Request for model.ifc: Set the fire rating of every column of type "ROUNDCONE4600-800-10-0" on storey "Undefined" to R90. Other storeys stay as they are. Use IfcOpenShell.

First a look at what the model holds.

```python
import ifcopenshell
import ifcopenshell.util.element

model = ifcopenshell.open("model.ifc")
print(model.schema)
storey = next(s for s in model.by_type("IfcBuildingStorey") if s.Name == "Undefined")
columns = [e for e in ifcopenshell.util.element.get_decomposition(storey) if e.is_a("IfcColumn")]
seen = {}
for e in columns:
    element_type = ifcopenshell.util.element.get_type(e)
    key = (element_type.Name if element_type != e and element_type else None, ifcopenshell.util.element.get_pset(e, "Pset_ColumnCommon", "FireRating"))
    seen[key] = seen.get(key, 0) + 1
for (name, value), count in sorted(seen.items(), key=str):
    print(count, "x", name, "|", value)
```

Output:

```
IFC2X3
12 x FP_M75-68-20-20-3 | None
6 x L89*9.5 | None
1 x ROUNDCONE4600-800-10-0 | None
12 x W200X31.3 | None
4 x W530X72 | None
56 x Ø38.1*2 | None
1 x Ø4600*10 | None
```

```python
import ifcopenshell
import ifcopenshell.api.pset
import ifcopenshell.util.element

model = ifcopenshell.open("model.ifc")

storey = next(s for s in model.by_type("IfcBuildingStorey") if s.Name == "Undefined")
columns = [e for e in ifcopenshell.util.element.get_decomposition(storey) if e.is_a("IfcColumn")]

count = 0
for e in columns:
    element_type = ifcopenshell.util.element.get_type(e)
    if element_type in (None, e) or element_type.Name != "ROUNDCONE4600-800-10-0":
        continue
    # add_pset returns the element's existing set when there is one.
    pset = ifcopenshell.api.pset.add_pset(model, product=e, name="Pset_ColumnCommon")
    ifcopenshell.api.pset.edit_pset(model, pset=pset, properties={"FireRating": "R90"})
    count += 1

print(count, "columns updated")

model.write("model_updated.ifc")
```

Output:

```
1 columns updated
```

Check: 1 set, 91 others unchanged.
